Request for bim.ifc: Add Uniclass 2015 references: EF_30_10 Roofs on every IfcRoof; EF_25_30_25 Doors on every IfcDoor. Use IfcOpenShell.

First a look at what the model holds.

```python
import ifcopenshell

model = ifcopenshell.open("bim.ifc")
print(model.schema)
print("classifications:", [c.Name for c in model.by_type("IfcClassification")])
for ifc_class in ("IfcDoor", "IfcRoof", "IfcStair", "IfcWall", "IfcWindow"):
    print(ifc_class, len(model.by_type(ifc_class)))
```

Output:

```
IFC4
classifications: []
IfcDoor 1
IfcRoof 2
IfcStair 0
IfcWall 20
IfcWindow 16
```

```python
import ifcopenshell
import ifcopenshell.api.classification

model = ifcopenshell.open("bim.ifc")

system = ifcopenshell.api.classification.add_classification(model, classification="Uniclass 2015")

codes = {
    "IfcRoof": ("EF_30_10", "Roofs"),
    "IfcDoor": ("EF_25_30_25", "Doors"),
}
for ifc_class, (code, name) in codes.items():
    products = model.by_type(ifc_class)
    ifcopenshell.api.classification.add_reference(
        model, products=products, classification=system, identification=code, name=name
    )
    print(code, len(products))

model.write("bim_edited.ifc")
```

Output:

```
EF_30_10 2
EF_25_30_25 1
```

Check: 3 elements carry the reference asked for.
